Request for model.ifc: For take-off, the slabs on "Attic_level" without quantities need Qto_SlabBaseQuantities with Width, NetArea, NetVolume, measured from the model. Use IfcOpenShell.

First a look at what the model holds.

```python
import ifcopenshell
import ifcopenshell.util.element
import ifcopenshell.util.unit

model = ifcopenshell.open("model.ifc")
print(model.schema)
for unit_type in ("LENGTHUNIT", "AREAUNIT", "VOLUMEUNIT"):
    print(unit_type, ifcopenshell.util.unit.calculate_unit_scale(model, unit_type))
storey = next(s for s in model.by_type("IfcBuildingStorey") if s.Name == "Attic_level")
slabs = [e for e in ifcopenshell.util.element.get_decomposition(storey) if e.is_a("IfcSlab")]
for e in sorted(slabs, key=lambda e: e.id()):
    print(e.id(), e.is_a(), e.Name, list(ifcopenshell.util.element.get_psets(e, qtos_only=True)), sep=" | ")
```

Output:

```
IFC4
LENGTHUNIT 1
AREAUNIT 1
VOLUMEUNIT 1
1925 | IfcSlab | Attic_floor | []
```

```python
import ifcopenshell
import ifcopenshell.api.pset
import ifcopenshell.geom
import ifcopenshell.util.element
import ifcopenshell.util.shape
import ifcopenshell.util.unit

model = ifcopenshell.open("model.ifc")
unit_scale = ifcopenshell.util.unit.calculate_unit_scale(model)
area_scale = ifcopenshell.util.unit.calculate_unit_scale(model, "AREAUNIT")
volume_scale = ifcopenshell.util.unit.calculate_unit_scale(model, "VOLUMEUNIT")
settings = ifcopenshell.geom.settings()

storey = next(s for s in model.by_type("IfcBuildingStorey") if s.Name == "Attic_level")
slabs = [e for e in ifcopenshell.util.element.get_decomposition(storey) if e.is_a("IfcSlab")]

for e in sorted(slabs, key=lambda e: e.id()):
    if ifcopenshell.util.element.get_psets(e, qtos_only=True, should_inherit=False):
        continue
    # Geometry comes back in metres, in the element's own axes.
    shape = ifcopenshell.geom.create_shape(settings, e)
    values = {
        "Width": ifcopenshell.util.shape.get_z(shape.geometry) / unit_scale,
        "NetArea": ifcopenshell.util.shape.get_footprint_area(shape.geometry) / area_scale,
        "NetVolume": ifcopenshell.util.shape.get_volume(shape.geometry) / volume_scale,
    }
    qto = ifcopenshell.api.pset.add_qto(model, product=e, name="Qto_SlabBaseQuantities")
    ifcopenshell.api.pset.edit_qto(model, qto=qto, properties=values)
    print(e.id(), {k: round(v, 3) for k, v in values.items()})

model.write("model-out.ifc")
```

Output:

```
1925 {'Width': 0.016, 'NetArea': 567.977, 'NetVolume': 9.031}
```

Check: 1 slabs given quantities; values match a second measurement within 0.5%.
